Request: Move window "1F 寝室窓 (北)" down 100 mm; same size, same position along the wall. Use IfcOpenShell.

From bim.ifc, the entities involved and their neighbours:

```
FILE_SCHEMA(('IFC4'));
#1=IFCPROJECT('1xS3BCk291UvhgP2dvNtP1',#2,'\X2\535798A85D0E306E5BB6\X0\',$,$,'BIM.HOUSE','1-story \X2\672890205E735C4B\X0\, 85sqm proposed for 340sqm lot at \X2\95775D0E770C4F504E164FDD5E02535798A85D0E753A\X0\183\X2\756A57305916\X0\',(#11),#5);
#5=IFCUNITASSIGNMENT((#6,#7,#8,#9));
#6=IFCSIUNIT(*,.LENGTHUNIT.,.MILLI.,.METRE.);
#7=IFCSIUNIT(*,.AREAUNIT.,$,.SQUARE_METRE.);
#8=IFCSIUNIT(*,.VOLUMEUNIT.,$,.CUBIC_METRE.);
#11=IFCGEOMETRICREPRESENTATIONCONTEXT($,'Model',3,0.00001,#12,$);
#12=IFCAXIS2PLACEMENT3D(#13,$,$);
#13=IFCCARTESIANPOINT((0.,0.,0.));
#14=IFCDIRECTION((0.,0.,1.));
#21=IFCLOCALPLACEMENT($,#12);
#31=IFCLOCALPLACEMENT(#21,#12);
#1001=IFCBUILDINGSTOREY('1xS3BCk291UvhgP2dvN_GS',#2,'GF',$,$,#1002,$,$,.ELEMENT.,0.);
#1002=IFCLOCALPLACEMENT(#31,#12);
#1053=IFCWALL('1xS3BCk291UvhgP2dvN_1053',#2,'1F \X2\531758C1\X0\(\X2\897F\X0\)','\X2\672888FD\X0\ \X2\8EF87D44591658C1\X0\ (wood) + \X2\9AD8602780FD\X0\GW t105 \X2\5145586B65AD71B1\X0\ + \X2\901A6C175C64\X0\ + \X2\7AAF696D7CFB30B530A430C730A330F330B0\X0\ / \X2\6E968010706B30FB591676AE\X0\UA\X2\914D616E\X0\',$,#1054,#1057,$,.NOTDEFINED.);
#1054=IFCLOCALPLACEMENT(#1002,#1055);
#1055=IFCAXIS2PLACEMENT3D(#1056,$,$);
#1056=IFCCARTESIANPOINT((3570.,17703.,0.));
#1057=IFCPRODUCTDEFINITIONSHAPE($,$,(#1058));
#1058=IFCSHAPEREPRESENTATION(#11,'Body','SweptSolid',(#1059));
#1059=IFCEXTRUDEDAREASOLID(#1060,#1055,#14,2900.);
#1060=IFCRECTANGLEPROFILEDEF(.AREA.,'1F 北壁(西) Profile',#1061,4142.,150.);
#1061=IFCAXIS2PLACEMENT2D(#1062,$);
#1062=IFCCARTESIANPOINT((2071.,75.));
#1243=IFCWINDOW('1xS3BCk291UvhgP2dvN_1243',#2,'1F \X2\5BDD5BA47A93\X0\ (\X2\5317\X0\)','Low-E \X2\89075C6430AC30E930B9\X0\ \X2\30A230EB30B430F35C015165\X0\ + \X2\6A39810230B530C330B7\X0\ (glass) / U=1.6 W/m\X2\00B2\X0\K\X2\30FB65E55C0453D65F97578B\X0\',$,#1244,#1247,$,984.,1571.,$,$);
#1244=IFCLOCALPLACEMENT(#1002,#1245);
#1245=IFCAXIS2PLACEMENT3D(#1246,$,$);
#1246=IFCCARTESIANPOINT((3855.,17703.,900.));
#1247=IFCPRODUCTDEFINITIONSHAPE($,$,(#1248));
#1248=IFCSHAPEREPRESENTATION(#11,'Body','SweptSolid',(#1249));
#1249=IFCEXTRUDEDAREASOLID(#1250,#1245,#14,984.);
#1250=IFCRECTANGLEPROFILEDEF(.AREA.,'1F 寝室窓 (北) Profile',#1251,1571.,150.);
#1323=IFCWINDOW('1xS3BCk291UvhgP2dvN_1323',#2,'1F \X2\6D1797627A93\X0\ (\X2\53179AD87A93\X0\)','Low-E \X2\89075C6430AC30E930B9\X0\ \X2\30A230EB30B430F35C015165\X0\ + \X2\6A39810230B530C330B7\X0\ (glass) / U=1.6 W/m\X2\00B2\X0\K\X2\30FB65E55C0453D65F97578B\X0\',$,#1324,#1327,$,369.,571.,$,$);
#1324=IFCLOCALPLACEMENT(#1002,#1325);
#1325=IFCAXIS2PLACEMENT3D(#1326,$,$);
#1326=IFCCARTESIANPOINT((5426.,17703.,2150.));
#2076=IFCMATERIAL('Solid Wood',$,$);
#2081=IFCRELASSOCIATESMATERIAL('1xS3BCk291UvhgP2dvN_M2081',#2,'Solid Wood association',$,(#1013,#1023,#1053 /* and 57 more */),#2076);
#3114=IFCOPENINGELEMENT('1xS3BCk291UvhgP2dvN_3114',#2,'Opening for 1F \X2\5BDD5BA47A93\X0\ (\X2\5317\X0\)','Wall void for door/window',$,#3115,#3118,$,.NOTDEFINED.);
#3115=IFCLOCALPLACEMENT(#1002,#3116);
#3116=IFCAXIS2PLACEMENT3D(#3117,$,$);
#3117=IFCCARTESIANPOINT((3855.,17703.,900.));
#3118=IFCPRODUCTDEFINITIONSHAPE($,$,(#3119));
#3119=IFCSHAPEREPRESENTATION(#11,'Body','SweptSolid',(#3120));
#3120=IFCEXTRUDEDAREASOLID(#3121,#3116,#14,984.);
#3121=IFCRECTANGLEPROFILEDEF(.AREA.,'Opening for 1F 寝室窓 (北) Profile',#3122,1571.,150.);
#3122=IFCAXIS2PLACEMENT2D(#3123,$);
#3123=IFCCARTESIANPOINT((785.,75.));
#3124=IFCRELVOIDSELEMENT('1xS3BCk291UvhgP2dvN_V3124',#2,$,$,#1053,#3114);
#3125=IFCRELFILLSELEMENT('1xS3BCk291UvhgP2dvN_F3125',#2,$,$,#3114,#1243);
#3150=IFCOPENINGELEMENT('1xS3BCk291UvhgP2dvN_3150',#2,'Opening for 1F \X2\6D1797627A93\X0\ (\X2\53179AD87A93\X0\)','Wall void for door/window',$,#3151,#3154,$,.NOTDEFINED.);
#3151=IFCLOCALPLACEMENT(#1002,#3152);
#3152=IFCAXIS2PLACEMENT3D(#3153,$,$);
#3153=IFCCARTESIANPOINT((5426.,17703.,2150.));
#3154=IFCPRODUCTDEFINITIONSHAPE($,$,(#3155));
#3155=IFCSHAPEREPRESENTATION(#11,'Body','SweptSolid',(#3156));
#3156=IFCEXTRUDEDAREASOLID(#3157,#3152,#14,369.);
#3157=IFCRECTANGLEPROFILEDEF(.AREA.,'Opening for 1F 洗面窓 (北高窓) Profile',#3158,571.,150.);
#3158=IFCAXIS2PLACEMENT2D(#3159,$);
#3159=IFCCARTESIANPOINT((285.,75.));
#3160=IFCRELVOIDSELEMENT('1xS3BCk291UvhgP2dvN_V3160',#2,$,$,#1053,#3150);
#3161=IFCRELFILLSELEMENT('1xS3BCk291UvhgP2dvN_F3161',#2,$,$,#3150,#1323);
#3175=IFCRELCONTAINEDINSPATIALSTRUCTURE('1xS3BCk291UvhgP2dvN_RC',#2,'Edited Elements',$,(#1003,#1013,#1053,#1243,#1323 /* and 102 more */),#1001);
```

```python
import numpy as np
import ifcopenshell
import ifcopenshell.api.geometry
import ifcopenshell.util.placement
import ifcopenshell.util.unit

model = ifcopenshell.open("bim.ifc")
unit_scale = ifcopenshell.util.unit.calculate_unit_scale(model)

window = model.by_id(1243)
opening = window.FillsVoids[0].RelatingOpeningElement
dz = -0.1 / unit_scale

shift = np.array([0.0, 0.0, dz])
# The window is not placed relative to its opening, so move both.
for product in (opening, window):
    matrix = ifcopenshell.util.placement.get_local_placement(product.ObjectPlacement)
    matrix[:3, 3] += shift
    ifcopenshell.api.geometry.edit_object_placement(model, product=product, matrix=matrix, is_si=False)

print(f"moved by {dz * unit_scale:+.3f} m")

model.write("bim-out.ifc")
```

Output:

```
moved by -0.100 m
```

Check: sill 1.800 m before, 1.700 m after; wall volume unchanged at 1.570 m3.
